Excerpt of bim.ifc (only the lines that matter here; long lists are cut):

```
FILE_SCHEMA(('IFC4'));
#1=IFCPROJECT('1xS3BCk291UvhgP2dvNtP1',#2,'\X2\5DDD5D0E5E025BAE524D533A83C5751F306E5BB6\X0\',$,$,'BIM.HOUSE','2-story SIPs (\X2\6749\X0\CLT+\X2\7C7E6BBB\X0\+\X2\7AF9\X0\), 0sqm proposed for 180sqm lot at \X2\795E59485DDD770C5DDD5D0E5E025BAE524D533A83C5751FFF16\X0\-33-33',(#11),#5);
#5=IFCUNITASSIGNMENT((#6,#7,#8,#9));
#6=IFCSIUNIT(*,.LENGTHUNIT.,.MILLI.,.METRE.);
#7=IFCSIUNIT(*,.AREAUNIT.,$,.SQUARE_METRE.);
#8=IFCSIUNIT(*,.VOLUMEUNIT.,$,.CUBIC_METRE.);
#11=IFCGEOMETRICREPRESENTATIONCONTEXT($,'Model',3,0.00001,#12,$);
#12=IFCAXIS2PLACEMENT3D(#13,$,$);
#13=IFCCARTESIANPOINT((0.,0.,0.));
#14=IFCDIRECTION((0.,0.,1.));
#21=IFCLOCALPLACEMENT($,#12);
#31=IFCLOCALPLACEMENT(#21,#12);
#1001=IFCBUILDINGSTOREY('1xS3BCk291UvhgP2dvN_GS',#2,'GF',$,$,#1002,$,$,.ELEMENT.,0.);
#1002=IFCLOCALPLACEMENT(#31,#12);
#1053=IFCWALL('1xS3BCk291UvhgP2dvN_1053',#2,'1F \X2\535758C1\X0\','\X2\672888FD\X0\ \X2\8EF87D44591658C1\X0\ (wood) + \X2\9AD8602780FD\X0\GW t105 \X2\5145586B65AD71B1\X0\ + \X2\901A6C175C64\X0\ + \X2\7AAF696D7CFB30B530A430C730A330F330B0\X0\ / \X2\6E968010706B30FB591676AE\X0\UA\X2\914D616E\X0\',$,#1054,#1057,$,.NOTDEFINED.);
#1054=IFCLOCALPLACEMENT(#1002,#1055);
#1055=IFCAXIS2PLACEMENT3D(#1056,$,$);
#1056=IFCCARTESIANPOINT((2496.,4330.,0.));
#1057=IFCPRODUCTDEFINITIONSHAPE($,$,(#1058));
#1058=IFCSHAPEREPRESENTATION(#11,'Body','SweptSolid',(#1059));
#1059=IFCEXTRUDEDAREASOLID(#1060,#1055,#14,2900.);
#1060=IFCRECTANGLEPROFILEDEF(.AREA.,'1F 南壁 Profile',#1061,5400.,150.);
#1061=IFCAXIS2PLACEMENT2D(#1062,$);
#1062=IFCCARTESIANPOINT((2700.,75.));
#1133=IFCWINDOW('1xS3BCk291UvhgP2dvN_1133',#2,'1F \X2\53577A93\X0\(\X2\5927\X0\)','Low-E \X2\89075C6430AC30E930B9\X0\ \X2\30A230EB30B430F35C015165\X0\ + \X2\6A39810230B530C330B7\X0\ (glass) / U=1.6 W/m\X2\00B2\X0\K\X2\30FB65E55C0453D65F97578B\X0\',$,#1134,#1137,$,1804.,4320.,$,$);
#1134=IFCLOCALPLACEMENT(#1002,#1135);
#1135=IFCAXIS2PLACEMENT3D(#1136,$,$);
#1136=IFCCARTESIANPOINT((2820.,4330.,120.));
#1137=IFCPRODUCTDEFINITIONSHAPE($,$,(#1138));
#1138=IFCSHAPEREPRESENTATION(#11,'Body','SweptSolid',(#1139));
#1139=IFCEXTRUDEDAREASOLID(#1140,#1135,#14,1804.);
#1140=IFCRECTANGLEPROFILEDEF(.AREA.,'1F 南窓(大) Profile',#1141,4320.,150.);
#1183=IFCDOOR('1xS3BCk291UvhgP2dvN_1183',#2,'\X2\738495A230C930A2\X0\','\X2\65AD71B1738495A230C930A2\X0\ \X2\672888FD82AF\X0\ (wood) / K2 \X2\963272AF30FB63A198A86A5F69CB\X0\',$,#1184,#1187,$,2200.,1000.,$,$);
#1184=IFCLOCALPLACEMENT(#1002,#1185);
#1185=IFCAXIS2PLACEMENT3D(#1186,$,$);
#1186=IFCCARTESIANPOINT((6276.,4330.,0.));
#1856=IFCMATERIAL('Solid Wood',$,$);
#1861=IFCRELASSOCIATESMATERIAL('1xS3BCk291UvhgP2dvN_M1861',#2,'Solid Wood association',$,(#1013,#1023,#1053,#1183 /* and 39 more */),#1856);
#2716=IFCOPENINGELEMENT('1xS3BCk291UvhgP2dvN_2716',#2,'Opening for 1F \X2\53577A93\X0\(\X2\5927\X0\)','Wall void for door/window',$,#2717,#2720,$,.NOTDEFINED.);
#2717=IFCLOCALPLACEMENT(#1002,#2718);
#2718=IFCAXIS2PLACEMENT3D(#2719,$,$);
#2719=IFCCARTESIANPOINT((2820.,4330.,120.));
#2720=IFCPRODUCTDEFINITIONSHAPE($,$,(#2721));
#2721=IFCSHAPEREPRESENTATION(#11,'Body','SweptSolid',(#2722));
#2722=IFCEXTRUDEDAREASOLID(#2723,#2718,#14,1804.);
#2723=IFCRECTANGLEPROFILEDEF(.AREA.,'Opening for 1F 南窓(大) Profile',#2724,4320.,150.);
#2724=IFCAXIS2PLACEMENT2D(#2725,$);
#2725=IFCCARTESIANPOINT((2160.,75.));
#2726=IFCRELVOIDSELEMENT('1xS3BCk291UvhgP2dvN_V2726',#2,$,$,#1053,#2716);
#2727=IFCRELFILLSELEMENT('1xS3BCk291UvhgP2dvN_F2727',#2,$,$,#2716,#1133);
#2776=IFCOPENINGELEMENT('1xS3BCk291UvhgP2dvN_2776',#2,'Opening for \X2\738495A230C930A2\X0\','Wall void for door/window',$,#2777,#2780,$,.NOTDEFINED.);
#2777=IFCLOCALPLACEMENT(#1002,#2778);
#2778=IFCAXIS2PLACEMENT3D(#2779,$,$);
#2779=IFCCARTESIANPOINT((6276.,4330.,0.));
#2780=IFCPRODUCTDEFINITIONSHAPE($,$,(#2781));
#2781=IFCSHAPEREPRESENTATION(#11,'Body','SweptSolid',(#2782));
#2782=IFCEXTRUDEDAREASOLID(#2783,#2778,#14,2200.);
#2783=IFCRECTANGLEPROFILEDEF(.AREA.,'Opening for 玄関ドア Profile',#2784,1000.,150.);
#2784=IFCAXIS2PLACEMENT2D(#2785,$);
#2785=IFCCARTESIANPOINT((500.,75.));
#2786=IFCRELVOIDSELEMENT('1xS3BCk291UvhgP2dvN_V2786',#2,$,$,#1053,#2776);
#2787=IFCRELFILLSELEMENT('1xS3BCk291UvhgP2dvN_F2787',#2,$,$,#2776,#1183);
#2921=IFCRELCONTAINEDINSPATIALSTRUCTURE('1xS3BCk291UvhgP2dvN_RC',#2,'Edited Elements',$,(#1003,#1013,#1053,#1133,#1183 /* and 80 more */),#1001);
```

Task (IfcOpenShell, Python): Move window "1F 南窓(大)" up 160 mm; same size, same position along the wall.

```python
import numpy as np
import ifcopenshell
import ifcopenshell.api.geometry
import ifcopenshell.util.placement
import ifcopenshell.util.unit

model = ifcopenshell.open("bim.ifc")
unit_scale = ifcopenshell.util.unit.calculate_unit_scale(model)

window = model.by_id(1133)
opening = window.FillsVoids[0].RelatingOpeningElement
dz = 0.16 / unit_scale

shift = np.array([0.0, 0.0, dz])
# The window is not placed relative to its opening, so move both.
for product in (opening, window):
    matrix = ifcopenshell.util.placement.get_local_placement(product.ObjectPlacement)
    matrix[:3, 3] += shift
    ifcopenshell.api.geometry.edit_object_placement(model, product=product, matrix=matrix, is_si=False)

print(f"moved by {dz * unit_scale:+.3f} m")

model.write("bim_updated.ifc")
```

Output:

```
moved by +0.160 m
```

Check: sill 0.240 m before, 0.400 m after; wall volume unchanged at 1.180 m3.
